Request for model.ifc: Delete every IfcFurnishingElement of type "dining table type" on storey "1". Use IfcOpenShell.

First a look at what the model holds.

```python
import ifcopenshell
import ifcopenshell.util.element

model = ifcopenshell.open("model.ifc")
print(model.schema)
storey = next(s for s in model.by_type("IfcBuildingStorey") if s.Name == "1")
furniture = [e for e in ifcopenshell.util.element.get_decomposition(storey) if e.is_a("IfcFurnishingElement")]
seen = {}
for e in furniture:
    element_type = ifcopenshell.util.element.get_type(e)
    name = element_type.Name if element_type not in (None, e) else None
    seen[name] = seen.get(name, 0) + 1
for name, count in sorted(seen.items(), key=str):
    print(count, "x", name)
```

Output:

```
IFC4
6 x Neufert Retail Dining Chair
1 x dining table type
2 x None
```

```python
import ifcopenshell
import ifcopenshell.api.root
import ifcopenshell.util.element

model = ifcopenshell.open("model.ifc")

storey = next(s for s in model.by_type("IfcBuildingStorey") if s.Name == "1")
furniture = [e for e in ifcopenshell.util.element.get_decomposition(storey) if e.is_a("IfcFurnishingElement")]
targets = [e for e in furniture if (t := ifcopenshell.util.element.get_type(e)) not in (None, e) and t.Name == "dining table type"]

for e in targets:
    ifcopenshell.api.root.remove_product(model, product=e)
print(len(targets), "removed")

model.write("model_updated.ifc")
```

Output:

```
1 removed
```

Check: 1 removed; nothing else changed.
